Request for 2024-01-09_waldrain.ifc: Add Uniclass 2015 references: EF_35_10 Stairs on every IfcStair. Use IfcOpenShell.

First a look at what the model holds.

```python
import ifcopenshell

model = ifcopenshell.open("2024-01-09_waldrain.ifc")
print(model.schema)
print("classifications:", [c.Name for c in model.by_type("IfcClassification")])
for ifc_class in ("IfcDoor", "IfcRoof", "IfcStair", "IfcWall", "IfcWindow"):
    print(ifc_class, len(model.by_type(ifc_class)))
```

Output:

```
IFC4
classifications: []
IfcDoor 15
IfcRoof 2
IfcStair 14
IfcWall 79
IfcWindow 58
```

```python
import ifcopenshell
import ifcopenshell.api.classification

model = ifcopenshell.open("2024-01-09_waldrain.ifc")

system = ifcopenshell.api.classification.add_classification(model, classification="Uniclass 2015")

codes = {
    "IfcStair": ("EF_35_10", "Stairs"),
}
for ifc_class, (code, name) in codes.items():
    products = model.by_type(ifc_class)
    ifcopenshell.api.classification.add_reference(
        model, products=products, classification=system, identification=code, name=name
    )
    print(code, len(products))

model.write("2024-01-09_waldrain_edited.ifc")
```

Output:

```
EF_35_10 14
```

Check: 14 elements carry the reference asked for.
